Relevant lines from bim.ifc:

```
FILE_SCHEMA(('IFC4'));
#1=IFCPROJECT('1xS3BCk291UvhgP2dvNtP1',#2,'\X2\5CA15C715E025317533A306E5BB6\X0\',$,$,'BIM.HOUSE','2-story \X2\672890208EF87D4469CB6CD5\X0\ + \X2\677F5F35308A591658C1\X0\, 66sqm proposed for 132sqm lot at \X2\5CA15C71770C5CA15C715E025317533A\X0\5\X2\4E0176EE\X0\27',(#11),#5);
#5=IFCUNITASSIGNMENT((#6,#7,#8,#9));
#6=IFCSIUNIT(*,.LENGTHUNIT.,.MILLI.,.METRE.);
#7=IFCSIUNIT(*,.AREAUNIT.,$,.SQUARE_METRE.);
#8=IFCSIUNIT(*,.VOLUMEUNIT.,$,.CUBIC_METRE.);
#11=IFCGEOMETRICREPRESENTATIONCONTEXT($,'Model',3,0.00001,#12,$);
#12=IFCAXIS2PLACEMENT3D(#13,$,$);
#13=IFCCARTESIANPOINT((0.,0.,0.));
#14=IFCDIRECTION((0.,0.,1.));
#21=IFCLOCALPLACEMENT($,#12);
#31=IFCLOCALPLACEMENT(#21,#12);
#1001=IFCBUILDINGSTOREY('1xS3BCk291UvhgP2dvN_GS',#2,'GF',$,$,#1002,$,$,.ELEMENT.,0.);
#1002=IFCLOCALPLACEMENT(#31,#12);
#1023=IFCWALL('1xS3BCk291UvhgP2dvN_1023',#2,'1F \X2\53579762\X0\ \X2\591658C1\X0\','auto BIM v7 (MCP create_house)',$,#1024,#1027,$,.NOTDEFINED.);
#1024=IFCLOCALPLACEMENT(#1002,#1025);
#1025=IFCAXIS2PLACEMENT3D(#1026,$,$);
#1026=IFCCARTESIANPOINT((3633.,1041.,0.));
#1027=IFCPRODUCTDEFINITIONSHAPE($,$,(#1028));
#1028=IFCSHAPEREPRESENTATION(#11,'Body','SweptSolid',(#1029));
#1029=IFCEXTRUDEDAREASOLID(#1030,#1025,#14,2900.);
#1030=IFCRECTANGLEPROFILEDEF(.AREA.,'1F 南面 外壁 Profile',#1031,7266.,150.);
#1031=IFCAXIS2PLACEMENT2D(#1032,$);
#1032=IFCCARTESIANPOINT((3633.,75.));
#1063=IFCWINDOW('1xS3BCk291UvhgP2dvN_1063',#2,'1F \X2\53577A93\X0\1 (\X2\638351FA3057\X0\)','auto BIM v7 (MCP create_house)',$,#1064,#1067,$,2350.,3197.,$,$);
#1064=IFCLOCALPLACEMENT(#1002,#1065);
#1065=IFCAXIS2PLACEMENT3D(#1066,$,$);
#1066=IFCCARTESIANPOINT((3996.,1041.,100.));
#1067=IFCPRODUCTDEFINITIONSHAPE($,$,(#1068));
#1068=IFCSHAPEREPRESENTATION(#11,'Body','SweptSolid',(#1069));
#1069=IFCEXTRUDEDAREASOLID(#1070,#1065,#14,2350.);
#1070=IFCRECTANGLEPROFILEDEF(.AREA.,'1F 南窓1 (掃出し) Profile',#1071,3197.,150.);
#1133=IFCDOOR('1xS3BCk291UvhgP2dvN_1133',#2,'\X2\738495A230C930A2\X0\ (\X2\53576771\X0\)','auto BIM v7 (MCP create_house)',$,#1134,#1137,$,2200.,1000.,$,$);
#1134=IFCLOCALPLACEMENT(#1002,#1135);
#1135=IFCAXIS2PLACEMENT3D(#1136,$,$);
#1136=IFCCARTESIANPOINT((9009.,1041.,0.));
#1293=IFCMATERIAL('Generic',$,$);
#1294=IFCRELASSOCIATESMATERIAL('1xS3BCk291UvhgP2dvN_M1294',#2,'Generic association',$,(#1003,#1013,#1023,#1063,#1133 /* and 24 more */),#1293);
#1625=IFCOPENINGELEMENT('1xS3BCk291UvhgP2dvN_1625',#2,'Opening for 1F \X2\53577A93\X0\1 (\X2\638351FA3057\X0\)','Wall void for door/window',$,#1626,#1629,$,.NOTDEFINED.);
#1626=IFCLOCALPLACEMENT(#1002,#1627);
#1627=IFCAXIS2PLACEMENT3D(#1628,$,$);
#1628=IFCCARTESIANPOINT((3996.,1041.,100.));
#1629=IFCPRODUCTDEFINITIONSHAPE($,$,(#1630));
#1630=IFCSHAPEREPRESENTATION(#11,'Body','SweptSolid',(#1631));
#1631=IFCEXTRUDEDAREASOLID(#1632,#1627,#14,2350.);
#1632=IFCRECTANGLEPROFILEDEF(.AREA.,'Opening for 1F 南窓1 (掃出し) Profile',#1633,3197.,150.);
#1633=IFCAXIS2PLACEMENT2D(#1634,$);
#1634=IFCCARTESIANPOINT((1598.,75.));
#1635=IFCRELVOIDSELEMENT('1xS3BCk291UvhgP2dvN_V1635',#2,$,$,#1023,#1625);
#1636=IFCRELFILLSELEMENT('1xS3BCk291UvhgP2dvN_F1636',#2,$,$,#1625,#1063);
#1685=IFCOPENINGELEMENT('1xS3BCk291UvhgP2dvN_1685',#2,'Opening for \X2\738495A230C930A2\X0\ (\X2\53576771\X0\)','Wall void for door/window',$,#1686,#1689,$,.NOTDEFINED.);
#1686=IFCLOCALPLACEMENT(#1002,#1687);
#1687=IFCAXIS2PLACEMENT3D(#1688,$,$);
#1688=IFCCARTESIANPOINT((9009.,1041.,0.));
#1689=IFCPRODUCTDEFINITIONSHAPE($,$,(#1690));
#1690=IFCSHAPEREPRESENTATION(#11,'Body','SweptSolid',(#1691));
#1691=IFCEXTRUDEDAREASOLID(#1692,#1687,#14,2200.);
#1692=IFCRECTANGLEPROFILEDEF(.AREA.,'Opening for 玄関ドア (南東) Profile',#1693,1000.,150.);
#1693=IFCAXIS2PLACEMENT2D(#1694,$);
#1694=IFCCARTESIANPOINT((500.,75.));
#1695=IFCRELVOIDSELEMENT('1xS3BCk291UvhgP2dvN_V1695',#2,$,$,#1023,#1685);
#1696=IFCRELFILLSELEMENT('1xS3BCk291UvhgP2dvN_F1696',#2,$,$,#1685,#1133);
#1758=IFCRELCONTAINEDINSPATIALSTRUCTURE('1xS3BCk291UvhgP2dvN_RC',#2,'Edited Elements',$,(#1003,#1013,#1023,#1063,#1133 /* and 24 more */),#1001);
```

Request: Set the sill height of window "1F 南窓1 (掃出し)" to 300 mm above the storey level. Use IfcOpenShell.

```python
import numpy as np
import ifcopenshell
import ifcopenshell.api.geometry
import ifcopenshell.geom
import ifcopenshell.util.element
import ifcopenshell.util.placement
import ifcopenshell.util.shape
import ifcopenshell.util.unit

model = ifcopenshell.open("bim.ifc")
unit_scale = ifcopenshell.util.unit.calculate_unit_scale(model)

window = model.by_guid("1xS3BCk291UvhgP2dvN_1063")
opening = window.FillsVoids[0].RelatingOpeningElement
storey = ifcopenshell.util.element.get_container(window, ifc_class="IfcBuildingStorey")
level = ifcopenshell.util.placement.get_local_placement(storey.ObjectPlacement)[2, 3]

# The opening's origin need not be at the sill, so measure its lowest point.
shape = ifcopenshell.geom.create_shape(ifcopenshell.geom.settings(), opening)
bottom = ifcopenshell.util.shape.get_shape_bottom_elevation(shape, shape.geometry) / unit_scale
dz = level + 0.3 / unit_scale - bottom

shift = np.array([0.0, 0.0, dz])
# The window is not placed relative to its opening, so move both.
for product in (opening, window):
    matrix = ifcopenshell.util.placement.get_local_placement(product.ObjectPlacement)
    matrix[:3, 3] += shift
    ifcopenshell.api.geometry.edit_object_placement(model, product=product, matrix=matrix, is_si=False)

print(f"moved by {dz * unit_scale:+.3f} m")

model.write("bim_v2.ifc")
```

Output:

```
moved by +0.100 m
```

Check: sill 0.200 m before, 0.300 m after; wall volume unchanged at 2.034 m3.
